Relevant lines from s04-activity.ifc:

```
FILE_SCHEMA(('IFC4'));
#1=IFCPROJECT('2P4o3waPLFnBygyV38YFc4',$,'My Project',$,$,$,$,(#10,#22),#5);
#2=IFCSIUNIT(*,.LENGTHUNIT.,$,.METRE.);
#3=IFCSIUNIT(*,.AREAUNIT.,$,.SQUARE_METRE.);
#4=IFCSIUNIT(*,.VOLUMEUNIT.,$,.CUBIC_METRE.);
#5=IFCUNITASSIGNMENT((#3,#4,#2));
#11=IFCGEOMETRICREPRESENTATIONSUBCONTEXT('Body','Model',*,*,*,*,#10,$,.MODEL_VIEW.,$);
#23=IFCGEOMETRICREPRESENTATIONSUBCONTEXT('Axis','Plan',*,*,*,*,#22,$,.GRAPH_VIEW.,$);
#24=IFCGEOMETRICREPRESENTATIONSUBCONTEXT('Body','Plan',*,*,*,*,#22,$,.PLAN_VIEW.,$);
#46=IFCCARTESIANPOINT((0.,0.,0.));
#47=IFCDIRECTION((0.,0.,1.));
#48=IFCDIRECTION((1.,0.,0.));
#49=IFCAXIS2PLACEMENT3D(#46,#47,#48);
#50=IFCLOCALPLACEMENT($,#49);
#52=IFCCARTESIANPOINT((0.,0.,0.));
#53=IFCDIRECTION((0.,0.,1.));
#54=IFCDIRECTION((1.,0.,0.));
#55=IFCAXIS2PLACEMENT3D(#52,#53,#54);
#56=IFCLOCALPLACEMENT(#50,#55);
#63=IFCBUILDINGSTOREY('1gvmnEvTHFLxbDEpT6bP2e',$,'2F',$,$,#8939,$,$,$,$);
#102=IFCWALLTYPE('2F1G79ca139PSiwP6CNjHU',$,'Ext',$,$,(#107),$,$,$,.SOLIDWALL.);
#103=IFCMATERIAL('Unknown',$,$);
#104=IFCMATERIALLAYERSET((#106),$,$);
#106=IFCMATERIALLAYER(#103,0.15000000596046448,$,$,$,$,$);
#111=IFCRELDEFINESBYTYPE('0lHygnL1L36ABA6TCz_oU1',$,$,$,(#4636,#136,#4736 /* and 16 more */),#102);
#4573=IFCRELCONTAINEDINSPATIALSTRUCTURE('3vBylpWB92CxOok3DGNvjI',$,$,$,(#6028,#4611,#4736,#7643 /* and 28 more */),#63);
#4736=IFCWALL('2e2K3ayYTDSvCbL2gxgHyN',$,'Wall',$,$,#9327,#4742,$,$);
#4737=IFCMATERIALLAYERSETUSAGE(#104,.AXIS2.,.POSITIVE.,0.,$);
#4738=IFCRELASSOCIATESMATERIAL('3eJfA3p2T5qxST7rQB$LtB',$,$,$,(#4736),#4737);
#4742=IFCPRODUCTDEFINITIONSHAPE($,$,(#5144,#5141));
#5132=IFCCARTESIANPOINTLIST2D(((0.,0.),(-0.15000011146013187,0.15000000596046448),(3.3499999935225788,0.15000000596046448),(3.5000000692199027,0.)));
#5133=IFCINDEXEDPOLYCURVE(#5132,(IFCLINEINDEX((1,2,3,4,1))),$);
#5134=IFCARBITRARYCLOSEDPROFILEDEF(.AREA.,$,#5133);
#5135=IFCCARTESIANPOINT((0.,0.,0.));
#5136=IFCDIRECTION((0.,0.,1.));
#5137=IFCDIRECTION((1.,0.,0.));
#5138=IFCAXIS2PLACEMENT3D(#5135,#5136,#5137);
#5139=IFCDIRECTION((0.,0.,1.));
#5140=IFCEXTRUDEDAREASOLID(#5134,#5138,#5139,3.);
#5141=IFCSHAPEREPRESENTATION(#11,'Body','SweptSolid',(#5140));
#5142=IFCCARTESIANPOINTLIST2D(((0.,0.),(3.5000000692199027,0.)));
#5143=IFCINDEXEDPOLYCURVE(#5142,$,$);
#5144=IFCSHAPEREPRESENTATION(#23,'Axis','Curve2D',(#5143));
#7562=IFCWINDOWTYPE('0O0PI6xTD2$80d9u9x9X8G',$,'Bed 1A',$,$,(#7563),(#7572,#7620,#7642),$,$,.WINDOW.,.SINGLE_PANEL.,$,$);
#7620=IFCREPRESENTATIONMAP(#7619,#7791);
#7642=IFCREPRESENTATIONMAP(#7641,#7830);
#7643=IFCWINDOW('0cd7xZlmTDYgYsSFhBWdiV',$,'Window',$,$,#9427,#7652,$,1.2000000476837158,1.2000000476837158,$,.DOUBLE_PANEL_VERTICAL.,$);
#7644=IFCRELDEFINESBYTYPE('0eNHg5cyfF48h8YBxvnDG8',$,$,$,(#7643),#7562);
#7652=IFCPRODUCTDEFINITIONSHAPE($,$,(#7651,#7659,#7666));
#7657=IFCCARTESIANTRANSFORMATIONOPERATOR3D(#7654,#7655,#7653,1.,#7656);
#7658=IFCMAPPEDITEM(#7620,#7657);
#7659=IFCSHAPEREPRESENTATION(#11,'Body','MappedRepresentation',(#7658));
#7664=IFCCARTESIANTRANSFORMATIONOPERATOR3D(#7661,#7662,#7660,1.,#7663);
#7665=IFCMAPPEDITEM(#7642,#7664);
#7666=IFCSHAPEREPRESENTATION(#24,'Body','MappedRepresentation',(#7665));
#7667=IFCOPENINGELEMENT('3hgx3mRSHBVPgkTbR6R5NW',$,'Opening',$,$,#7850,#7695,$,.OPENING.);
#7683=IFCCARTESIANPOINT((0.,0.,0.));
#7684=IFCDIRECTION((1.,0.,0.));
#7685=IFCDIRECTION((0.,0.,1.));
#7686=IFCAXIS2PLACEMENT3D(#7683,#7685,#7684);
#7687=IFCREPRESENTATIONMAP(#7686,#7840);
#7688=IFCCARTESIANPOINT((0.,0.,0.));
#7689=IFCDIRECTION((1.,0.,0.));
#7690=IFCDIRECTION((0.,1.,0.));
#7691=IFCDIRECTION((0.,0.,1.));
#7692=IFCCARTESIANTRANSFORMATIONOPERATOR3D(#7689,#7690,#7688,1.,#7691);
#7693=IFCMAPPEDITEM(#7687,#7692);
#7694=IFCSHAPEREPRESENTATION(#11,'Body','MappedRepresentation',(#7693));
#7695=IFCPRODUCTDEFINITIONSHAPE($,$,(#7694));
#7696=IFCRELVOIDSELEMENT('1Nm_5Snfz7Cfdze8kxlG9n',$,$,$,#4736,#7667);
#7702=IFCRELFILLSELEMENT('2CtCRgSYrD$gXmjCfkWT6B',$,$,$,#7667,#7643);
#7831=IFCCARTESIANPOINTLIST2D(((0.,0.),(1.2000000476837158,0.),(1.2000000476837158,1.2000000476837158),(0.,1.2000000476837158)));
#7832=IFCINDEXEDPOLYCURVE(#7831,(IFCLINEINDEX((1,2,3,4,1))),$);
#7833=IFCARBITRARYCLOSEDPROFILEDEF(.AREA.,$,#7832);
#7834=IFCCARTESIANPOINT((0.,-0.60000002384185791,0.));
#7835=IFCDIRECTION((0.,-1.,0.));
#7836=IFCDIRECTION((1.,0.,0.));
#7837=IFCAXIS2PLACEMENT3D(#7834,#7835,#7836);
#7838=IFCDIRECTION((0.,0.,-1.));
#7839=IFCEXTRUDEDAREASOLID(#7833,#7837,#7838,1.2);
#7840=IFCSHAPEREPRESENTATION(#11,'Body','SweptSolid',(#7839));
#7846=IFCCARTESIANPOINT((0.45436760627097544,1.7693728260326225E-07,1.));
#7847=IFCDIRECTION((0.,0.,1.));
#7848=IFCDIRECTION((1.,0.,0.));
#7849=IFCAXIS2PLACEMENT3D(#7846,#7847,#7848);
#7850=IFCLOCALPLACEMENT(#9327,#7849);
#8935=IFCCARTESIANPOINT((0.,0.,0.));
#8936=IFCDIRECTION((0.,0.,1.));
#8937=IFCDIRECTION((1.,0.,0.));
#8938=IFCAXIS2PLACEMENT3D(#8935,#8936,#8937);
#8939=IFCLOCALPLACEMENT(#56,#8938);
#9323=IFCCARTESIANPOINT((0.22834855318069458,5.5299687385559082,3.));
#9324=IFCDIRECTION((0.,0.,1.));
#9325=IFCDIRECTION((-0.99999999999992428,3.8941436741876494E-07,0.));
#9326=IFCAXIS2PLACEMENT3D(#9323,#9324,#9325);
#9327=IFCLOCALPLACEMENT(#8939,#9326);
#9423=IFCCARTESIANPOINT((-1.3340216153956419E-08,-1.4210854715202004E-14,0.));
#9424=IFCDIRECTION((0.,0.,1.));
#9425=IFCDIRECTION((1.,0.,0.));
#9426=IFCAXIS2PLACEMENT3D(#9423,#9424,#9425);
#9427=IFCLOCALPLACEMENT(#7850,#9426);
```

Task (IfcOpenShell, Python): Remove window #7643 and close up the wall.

```python
import ifcopenshell
import ifcopenshell.api.feature
import ifcopenshell.api.root
import ifcopenshell.geom
import ifcopenshell.util.shape

model = ifcopenshell.open("s04-activity.ifc")
settings = ifcopenshell.geom.settings()


def volume(element):
    """Net volume in cubic metres, openings subtracted."""
    shape = ifcopenshell.geom.create_shape(settings, element)
    return ifcopenshell.util.shape.get_volume(shape.geometry)


window = model.by_guid("0cd7xZlmTDYgYsSFhBWdiV")
opening = window.FillsVoids[0].RelatingOpeningElement
wall = opening.VoidsElements[0].RelatingBuildingElement
before = volume(wall)

ifcopenshell.api.root.remove_product(model, product=window)
ifcopenshell.api.feature.remove_feature(model, feature=opening)

after = volume(wall)

print(f"wall volume {before:.3f} -> {after:.3f} m3")

model.write("s04-activity_updated.ifc")
```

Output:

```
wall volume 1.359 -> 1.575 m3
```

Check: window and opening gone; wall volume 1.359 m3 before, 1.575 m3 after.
